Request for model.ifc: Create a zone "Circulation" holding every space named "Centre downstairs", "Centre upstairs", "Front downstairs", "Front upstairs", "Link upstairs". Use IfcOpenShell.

First a look at what the model holds.

```python
import ifcopenshell

model = ifcopenshell.open("model.ifc")
print(model.schema)
seen = {}
for space in model.by_type("IfcSpace"):
    seen[space.Name] = seen.get(space.Name, 0) + 1
for name, count in sorted(seen.items(), key=str):
    print(count, "x", name)
print("zones:", [z.Name for z in model.by_type("IfcZone")][:20])
```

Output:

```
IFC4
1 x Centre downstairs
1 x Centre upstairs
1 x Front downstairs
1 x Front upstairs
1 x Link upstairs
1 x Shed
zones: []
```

```python
import ifcopenshell
import ifcopenshell.api.group
import ifcopenshell.api.root

model = ifcopenshell.open("model.ifc")

names = {"Centre downstairs", "Centre upstairs", "Front downstairs", "Front upstairs", "Link upstairs"}
spaces = [s for s in model.by_type("IfcSpace") if s.Name in names]

zone = ifcopenshell.api.root.create_entity(model, ifc_class="IfcZone", name="Circulation")
ifcopenshell.api.group.assign_group(model, products=spaces, group=zone)
print(len(spaces), "spaces in", zone.Name)

model.write("model_v2.ifc")
```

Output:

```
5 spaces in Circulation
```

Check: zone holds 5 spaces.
